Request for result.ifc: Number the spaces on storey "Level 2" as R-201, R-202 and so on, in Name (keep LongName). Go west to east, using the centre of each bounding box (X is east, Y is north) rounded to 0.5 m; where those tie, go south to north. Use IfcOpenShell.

First a look at what the model holds.

```python
import ifcopenshell
import ifcopenshell.util.element
import ifcopenshell.util.placement

model = ifcopenshell.open("result.ifc")
print(model.schema)
storey = next(s for s in model.by_type("IfcBuildingStorey") if s.Name == "Level 2")
spaces = [e for e in ifcopenshell.util.element.get_decomposition(storey) if e.is_a("IfcSpace")]
for e in sorted(spaces, key=lambda e: e.id()):
    origin = ifcopenshell.util.placement.get_local_placement(e.ObjectPlacement)[:3, 3]
    print(e.id(), e.Name, e.LongName, origin.round(2) + 0.0, sep=" | ")
```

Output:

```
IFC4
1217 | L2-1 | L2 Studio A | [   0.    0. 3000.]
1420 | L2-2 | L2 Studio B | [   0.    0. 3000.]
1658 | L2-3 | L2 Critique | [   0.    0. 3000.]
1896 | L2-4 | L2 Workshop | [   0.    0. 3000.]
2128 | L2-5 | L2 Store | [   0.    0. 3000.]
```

```python
import ifcopenshell
import ifcopenshell.geom
import ifcopenshell.util.element
import ifcopenshell.util.shape

model = ifcopenshell.open("result.ifc")
settings = ifcopenshell.geom.settings()
settings.set("use-world-coords", True)


def centre(element):
    shape = ifcopenshell.geom.create_shape(settings, element)
    return ifcopenshell.util.shape.get_bbox_centroid(shape.geometry)


storey = next(s for s in model.by_type("IfcBuildingStorey") if s.Name == "Level 2")
spaces = [e for e in ifcopenshell.util.element.get_decomposition(storey) if e.is_a("IfcSpace")]

# Insertion points can sit at a corner or the storey origin, so sort by the geometry (in metres).
centres = {e: centre(e) for e in spaces}
spaces.sort(key=lambda e: (round(centres[e][0] / 0.5), centres[e][1]))

for i, e in enumerate(spaces, start=1):
    number = f"R-2{i:02d}"
    e.Name = number
    print(e.id(), number)

model.write("result-out.ifc")
```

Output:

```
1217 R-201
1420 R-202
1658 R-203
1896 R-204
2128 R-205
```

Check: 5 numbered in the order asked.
